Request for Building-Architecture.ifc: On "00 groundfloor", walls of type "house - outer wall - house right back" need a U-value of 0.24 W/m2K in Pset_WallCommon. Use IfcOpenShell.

First a look at what the model holds.

```python
import ifcopenshell
import ifcopenshell.util.element

model = ifcopenshell.open("Building-Architecture.ifc")
print(model.schema)
storey = next(s for s in model.by_type("IfcBuildingStorey") if s.Name == "00 groundfloor")
walls = [e for e in ifcopenshell.util.element.get_decomposition(storey) if e.is_a("IfcWall")]
seen = {}
for e in walls:
    element_type = ifcopenshell.util.element.get_type(e)
    key = (element_type.Name if element_type != e and element_type else None, ifcopenshell.util.element.get_pset(e, "Pset_WallCommon", "ThermalTransmittance"))
    seen[key] = seen.get(key, 0) + 1
for (name, value), count in sorted(seen.items(), key=str):
    print(count, "x", name, "|", value)
```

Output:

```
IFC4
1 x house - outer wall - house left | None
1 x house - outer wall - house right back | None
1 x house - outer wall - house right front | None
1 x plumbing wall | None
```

```python
import ifcopenshell
import ifcopenshell.api.pset
import ifcopenshell.util.element

model = ifcopenshell.open("Building-Architecture.ifc")

storey = next(s for s in model.by_type("IfcBuildingStorey") if s.Name == "00 groundfloor")
walls = [e for e in ifcopenshell.util.element.get_decomposition(storey) if e.is_a("IfcWall")]

count = 0
for e in walls:
    element_type = ifcopenshell.util.element.get_type(e)
    if element_type in (None, e) or element_type.Name != "house - outer wall - house right back":
        continue
    # add_pset returns the element's existing set when there is one.
    pset = ifcopenshell.api.pset.add_pset(model, product=e, name="Pset_WallCommon")
    ifcopenshell.api.pset.edit_pset(model, pset=pset, properties={"ThermalTransmittance": 0.24})
    count += 1

print(count, "walls updated")

model.write("Building-Architecture_edited.ifc")
```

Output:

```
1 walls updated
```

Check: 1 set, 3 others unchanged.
